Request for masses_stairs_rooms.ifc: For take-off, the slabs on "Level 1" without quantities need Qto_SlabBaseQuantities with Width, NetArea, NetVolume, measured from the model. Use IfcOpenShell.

First a look at what the model holds.

```python
import ifcopenshell
import ifcopenshell.util.element
import ifcopenshell.util.unit

model = ifcopenshell.open("masses_stairs_rooms.ifc")
print(model.schema)
for unit_type in ("LENGTHUNIT", "AREAUNIT", "VOLUMEUNIT"):
    print(unit_type, ifcopenshell.util.unit.calculate_unit_scale(model, unit_type))
storey = next(s for s in model.by_type("IfcBuildingStorey") if s.Name == "Level 1")
slabs = [e for e in ifcopenshell.util.element.get_decomposition(storey) if e.is_a("IfcSlab")]
for e in sorted(slabs, key=lambda e: e.id()):
    print(e.id(), e.is_a(), e.Name, list(ifcopenshell.util.element.get_psets(e, qtos_only=True)), sep=" | ")
```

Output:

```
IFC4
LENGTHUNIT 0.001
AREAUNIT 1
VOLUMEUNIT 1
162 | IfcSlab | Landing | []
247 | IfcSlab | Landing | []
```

```python
import ifcopenshell
import ifcopenshell.api.pset
import ifcopenshell.geom
import ifcopenshell.util.element
import ifcopenshell.util.shape
import ifcopenshell.util.unit

model = ifcopenshell.open("masses_stairs_rooms.ifc")
unit_scale = ifcopenshell.util.unit.calculate_unit_scale(model)
area_scale = ifcopenshell.util.unit.calculate_unit_scale(model, "AREAUNIT")
volume_scale = ifcopenshell.util.unit.calculate_unit_scale(model, "VOLUMEUNIT")
settings = ifcopenshell.geom.settings()

storey = next(s for s in model.by_type("IfcBuildingStorey") if s.Name == "Level 1")
slabs = [e for e in ifcopenshell.util.element.get_decomposition(storey) if e.is_a("IfcSlab")]

for e in sorted(slabs, key=lambda e: e.id()):
    if ifcopenshell.util.element.get_psets(e, qtos_only=True, should_inherit=False):
        continue
    # Geometry comes back in metres, in the element's own axes.
    shape = ifcopenshell.geom.create_shape(settings, e)
    values = {
        "Width": ifcopenshell.util.shape.get_z(shape.geometry) / unit_scale,
        "NetArea": ifcopenshell.util.shape.get_footprint_area(shape.geometry) / area_scale,
        "NetVolume": ifcopenshell.util.shape.get_volume(shape.geometry) / volume_scale,
    }
    qto = ifcopenshell.api.pset.add_qto(model, product=e, name="Qto_SlabBaseQuantities")
    ifcopenshell.api.pset.edit_qto(model, qto=qto, properties=values)
    print(e.id(), {k: round(v, 3) for k, v in values.items()})

model.write("masses_stairs_rooms_v2.ifc")
```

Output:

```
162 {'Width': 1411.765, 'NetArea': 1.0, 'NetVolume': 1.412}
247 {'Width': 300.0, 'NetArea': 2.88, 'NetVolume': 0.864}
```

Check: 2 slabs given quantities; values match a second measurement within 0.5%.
